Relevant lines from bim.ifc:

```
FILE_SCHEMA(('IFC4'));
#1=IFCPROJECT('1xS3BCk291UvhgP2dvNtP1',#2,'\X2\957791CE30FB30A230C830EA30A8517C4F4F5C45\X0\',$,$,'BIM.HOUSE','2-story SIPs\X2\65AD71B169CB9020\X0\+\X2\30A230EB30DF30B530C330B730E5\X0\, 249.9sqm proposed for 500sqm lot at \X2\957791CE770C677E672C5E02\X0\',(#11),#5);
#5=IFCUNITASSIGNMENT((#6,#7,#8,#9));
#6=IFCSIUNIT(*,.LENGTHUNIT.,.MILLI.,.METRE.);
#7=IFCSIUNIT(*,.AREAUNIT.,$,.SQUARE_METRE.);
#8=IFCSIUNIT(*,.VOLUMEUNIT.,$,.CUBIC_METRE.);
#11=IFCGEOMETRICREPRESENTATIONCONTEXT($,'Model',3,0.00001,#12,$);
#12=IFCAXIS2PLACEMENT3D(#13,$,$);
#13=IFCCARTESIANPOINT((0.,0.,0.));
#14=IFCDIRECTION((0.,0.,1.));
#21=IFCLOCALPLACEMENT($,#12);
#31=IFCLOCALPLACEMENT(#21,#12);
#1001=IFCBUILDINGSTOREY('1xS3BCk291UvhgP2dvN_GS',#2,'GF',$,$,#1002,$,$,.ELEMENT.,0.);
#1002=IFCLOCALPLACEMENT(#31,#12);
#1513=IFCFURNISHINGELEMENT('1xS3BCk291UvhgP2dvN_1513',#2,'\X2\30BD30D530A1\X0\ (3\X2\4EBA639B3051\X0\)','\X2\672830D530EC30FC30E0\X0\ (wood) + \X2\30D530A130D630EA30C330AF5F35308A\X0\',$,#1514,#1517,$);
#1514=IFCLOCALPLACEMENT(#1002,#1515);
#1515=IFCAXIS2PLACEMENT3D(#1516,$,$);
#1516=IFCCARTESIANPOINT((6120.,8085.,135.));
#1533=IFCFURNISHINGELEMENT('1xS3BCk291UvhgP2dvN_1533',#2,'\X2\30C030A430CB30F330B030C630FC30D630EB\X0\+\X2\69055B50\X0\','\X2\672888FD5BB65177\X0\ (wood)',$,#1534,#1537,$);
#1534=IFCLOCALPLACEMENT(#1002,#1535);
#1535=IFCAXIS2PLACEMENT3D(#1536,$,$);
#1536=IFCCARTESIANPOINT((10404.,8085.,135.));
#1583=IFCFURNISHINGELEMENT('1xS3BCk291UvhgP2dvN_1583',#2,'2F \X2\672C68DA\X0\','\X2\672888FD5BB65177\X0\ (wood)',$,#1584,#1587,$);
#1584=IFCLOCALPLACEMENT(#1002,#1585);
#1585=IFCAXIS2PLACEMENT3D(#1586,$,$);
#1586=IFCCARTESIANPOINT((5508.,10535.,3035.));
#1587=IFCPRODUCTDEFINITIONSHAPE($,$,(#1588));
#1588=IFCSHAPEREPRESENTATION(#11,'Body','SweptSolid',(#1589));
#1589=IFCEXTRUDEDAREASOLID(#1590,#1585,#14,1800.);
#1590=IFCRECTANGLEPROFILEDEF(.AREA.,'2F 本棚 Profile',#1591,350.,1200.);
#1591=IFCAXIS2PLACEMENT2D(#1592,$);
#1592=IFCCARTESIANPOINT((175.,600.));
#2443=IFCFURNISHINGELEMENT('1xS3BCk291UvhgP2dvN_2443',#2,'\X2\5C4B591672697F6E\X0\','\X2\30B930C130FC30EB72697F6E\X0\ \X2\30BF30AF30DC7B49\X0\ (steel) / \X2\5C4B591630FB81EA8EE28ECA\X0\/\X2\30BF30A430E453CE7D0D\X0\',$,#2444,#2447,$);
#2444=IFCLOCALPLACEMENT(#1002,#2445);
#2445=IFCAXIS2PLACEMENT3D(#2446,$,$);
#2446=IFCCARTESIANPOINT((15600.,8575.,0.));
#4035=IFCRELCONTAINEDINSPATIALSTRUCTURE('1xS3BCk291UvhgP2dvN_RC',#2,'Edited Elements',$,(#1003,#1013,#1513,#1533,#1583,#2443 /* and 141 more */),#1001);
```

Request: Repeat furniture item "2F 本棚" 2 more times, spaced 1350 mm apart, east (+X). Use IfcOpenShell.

```python
import numpy as np
import ifcopenshell
import ifcopenshell.api.geometry
import ifcopenshell.api.root
import ifcopenshell.util.element
import ifcopenshell.util.placement
import ifcopenshell.util.unit

model = ifcopenshell.open("bim.ifc")
unit_scale = ifcopenshell.util.unit.calculate_unit_scale(model)


def reuse_history(source, copy):
    """copy_class also copies each property set's owner history, people and application; keep the originals."""
    for rel in copy.IsDefinedBy:
        if rel.is_a("IfcRelDefinesByProperties") and (history := rel.RelatingPropertyDefinition.OwnerHistory):
            rel.RelatingPropertyDefinition.OwnerHistory = source.OwnerHistory
            ifcopenshell.util.element.remove_deep2(model, history)


source = model.by_guid("1xS3BCk291UvhgP2dvN_1583")
base = ifcopenshell.util.placement.get_local_placement(source.ObjectPlacement)
step = np.array([1.0, 0.0, 0.0]) * 1.35 / unit_scale

for i in range(1, 3):
    copy = ifcopenshell.api.root.copy_class(model, product=source)
    copy.Representation = ifcopenshell.util.element.copy_deep(
        model, source.Representation, exclude=["IfcGeometricRepresentationContext", "IfcRepresentationMap"]
    )
    reuse_history(source, copy)
    matrix = base.copy()
    matrix[:3, 3] += i * step
    print("added at", matrix[:3, 3].round(3) + 0.0)
    ifcopenshell.api.geometry.edit_object_placement(model, product=copy, matrix=matrix, is_si=False)

model.write("bim_updated.ifc")
```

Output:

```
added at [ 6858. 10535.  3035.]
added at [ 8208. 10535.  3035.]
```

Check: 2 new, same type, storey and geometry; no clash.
